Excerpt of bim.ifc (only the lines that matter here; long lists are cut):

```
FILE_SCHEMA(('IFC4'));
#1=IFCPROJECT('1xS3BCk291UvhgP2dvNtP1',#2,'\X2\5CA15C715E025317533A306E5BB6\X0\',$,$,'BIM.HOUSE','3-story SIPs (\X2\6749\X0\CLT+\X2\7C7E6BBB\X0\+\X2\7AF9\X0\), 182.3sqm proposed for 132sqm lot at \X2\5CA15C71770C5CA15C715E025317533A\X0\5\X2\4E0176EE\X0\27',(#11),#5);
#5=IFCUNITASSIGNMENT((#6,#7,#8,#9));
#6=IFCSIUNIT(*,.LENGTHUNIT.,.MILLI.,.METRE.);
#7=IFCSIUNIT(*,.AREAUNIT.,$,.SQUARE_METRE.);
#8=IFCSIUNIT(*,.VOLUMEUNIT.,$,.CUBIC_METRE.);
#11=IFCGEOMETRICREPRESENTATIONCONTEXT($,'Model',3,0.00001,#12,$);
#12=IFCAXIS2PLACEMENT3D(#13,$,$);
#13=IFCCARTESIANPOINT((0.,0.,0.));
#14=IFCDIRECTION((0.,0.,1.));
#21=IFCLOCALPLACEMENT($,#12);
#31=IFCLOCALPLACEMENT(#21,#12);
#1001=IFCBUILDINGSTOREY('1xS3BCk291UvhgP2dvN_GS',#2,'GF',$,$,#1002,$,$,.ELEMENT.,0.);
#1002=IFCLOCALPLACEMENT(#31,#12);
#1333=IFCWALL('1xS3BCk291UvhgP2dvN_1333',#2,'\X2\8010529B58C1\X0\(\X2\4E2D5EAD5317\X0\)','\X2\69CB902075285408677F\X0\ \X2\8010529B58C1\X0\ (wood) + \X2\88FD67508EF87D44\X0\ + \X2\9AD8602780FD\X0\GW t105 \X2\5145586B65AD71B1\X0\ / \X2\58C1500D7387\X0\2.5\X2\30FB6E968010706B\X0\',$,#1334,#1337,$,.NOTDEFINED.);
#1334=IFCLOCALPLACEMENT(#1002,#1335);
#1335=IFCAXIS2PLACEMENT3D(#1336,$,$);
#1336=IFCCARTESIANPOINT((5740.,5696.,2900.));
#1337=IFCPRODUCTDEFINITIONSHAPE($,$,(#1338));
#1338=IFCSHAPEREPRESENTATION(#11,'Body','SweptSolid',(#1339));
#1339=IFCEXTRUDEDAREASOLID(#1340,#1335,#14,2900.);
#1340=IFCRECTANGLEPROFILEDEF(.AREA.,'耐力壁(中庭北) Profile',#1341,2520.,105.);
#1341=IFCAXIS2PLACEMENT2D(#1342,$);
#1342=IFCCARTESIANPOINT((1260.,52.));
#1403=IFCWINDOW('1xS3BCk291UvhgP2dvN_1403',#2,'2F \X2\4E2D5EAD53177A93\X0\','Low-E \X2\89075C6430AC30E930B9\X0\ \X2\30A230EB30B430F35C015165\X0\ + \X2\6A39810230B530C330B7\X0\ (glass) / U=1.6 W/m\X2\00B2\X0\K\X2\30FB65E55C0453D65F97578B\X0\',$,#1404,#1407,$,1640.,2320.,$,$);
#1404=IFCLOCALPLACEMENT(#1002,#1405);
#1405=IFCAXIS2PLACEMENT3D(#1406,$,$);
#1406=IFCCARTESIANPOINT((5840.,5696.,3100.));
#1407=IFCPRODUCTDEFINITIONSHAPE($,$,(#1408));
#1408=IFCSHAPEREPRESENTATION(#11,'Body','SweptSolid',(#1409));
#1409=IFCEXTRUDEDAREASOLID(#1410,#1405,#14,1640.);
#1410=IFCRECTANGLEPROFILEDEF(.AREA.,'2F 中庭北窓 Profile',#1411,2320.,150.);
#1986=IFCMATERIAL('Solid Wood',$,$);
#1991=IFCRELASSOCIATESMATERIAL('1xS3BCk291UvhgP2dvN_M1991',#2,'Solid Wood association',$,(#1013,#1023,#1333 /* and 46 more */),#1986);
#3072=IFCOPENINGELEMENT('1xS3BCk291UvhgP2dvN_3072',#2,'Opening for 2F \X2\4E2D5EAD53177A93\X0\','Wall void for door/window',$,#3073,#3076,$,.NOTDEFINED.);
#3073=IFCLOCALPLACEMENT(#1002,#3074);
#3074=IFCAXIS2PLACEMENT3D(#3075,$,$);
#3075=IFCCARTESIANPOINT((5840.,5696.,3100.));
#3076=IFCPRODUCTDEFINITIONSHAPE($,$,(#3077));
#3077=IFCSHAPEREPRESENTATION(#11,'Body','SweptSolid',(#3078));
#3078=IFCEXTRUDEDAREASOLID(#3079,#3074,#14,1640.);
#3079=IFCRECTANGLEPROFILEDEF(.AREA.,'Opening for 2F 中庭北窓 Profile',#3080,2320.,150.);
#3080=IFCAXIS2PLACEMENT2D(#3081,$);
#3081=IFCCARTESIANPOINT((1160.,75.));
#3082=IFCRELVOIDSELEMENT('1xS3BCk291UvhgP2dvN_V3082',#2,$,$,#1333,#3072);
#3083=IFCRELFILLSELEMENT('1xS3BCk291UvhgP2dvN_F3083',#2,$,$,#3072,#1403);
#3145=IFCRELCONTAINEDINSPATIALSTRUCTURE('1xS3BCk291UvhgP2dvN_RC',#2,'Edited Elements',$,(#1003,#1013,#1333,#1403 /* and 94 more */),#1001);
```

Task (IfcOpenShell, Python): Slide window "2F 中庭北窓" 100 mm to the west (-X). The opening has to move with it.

```python
import ifcopenshell
import ifcopenshell.api.geometry
import ifcopenshell.util.placement
import ifcopenshell.util.unit

model = ifcopenshell.open("bim.ifc")
unit_scale = ifcopenshell.util.unit.calculate_unit_scale(model)

window = model.by_guid("1xS3BCk291UvhgP2dvN_1403")
opening = window.FillsVoids[0].RelatingOpeningElement
wall = opening.VoidsElements[0].RelatingBuildingElement

wall_matrix = ifcopenshell.util.placement.get_local_placement(wall.ObjectPlacement)
shift = wall_matrix[:3, 0] * -0.1 / unit_scale
before = ifcopenshell.util.placement.get_local_placement(window.ObjectPlacement)[:3, 3].copy()

# The window is not placed relative to its opening, so move both.
for product in (opening, window):
    matrix = ifcopenshell.util.placement.get_local_placement(product.ObjectPlacement)
    matrix[:3, 3] += shift
    ifcopenshell.api.geometry.edit_object_placement(model, product=product, matrix=matrix, is_si=False)

after = ifcopenshell.util.placement.get_local_placement(window.ObjectPlacement)[:3, 3]
print("window moved by", (after - before).round(3) + 0.0)

model.write("bim_v2.ifc")
```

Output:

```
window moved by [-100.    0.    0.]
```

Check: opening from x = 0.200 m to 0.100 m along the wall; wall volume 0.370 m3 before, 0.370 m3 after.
